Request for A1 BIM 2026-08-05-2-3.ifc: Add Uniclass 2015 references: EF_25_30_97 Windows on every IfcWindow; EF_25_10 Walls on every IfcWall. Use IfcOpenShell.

First a look at what the model holds.

```python
import ifcopenshell

model = ifcopenshell.open("A1 BIM 2026-08-05-2-3.ifc")
print(model.schema)
print("classifications:", [c.Name for c in model.by_type("IfcClassification")])
for ifc_class in ("IfcDoor", "IfcRoof", "IfcStair", "IfcWall", "IfcWindow"):
    print(ifc_class, len(model.by_type(ifc_class)))
```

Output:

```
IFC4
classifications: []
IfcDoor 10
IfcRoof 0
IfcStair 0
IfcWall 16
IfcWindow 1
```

```python
import ifcopenshell
import ifcopenshell.api.classification

model = ifcopenshell.open("A1 BIM 2026-08-05-2-3.ifc")

system = ifcopenshell.api.classification.add_classification(model, classification="Uniclass 2015")

codes = {
    "IfcWindow": ("EF_25_30_97", "Windows"),
    "IfcWall": ("EF_25_10", "Walls"),
}
for ifc_class, (code, name) in codes.items():
    products = model.by_type(ifc_class)
    ifcopenshell.api.classification.add_reference(
        model, products=products, classification=system, identification=code, name=name
    )
    print(code, len(products))

model.write("A1 BIM 2026-08-05-2-3_rev.ifc")
```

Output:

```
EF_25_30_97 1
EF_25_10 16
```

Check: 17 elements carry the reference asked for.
